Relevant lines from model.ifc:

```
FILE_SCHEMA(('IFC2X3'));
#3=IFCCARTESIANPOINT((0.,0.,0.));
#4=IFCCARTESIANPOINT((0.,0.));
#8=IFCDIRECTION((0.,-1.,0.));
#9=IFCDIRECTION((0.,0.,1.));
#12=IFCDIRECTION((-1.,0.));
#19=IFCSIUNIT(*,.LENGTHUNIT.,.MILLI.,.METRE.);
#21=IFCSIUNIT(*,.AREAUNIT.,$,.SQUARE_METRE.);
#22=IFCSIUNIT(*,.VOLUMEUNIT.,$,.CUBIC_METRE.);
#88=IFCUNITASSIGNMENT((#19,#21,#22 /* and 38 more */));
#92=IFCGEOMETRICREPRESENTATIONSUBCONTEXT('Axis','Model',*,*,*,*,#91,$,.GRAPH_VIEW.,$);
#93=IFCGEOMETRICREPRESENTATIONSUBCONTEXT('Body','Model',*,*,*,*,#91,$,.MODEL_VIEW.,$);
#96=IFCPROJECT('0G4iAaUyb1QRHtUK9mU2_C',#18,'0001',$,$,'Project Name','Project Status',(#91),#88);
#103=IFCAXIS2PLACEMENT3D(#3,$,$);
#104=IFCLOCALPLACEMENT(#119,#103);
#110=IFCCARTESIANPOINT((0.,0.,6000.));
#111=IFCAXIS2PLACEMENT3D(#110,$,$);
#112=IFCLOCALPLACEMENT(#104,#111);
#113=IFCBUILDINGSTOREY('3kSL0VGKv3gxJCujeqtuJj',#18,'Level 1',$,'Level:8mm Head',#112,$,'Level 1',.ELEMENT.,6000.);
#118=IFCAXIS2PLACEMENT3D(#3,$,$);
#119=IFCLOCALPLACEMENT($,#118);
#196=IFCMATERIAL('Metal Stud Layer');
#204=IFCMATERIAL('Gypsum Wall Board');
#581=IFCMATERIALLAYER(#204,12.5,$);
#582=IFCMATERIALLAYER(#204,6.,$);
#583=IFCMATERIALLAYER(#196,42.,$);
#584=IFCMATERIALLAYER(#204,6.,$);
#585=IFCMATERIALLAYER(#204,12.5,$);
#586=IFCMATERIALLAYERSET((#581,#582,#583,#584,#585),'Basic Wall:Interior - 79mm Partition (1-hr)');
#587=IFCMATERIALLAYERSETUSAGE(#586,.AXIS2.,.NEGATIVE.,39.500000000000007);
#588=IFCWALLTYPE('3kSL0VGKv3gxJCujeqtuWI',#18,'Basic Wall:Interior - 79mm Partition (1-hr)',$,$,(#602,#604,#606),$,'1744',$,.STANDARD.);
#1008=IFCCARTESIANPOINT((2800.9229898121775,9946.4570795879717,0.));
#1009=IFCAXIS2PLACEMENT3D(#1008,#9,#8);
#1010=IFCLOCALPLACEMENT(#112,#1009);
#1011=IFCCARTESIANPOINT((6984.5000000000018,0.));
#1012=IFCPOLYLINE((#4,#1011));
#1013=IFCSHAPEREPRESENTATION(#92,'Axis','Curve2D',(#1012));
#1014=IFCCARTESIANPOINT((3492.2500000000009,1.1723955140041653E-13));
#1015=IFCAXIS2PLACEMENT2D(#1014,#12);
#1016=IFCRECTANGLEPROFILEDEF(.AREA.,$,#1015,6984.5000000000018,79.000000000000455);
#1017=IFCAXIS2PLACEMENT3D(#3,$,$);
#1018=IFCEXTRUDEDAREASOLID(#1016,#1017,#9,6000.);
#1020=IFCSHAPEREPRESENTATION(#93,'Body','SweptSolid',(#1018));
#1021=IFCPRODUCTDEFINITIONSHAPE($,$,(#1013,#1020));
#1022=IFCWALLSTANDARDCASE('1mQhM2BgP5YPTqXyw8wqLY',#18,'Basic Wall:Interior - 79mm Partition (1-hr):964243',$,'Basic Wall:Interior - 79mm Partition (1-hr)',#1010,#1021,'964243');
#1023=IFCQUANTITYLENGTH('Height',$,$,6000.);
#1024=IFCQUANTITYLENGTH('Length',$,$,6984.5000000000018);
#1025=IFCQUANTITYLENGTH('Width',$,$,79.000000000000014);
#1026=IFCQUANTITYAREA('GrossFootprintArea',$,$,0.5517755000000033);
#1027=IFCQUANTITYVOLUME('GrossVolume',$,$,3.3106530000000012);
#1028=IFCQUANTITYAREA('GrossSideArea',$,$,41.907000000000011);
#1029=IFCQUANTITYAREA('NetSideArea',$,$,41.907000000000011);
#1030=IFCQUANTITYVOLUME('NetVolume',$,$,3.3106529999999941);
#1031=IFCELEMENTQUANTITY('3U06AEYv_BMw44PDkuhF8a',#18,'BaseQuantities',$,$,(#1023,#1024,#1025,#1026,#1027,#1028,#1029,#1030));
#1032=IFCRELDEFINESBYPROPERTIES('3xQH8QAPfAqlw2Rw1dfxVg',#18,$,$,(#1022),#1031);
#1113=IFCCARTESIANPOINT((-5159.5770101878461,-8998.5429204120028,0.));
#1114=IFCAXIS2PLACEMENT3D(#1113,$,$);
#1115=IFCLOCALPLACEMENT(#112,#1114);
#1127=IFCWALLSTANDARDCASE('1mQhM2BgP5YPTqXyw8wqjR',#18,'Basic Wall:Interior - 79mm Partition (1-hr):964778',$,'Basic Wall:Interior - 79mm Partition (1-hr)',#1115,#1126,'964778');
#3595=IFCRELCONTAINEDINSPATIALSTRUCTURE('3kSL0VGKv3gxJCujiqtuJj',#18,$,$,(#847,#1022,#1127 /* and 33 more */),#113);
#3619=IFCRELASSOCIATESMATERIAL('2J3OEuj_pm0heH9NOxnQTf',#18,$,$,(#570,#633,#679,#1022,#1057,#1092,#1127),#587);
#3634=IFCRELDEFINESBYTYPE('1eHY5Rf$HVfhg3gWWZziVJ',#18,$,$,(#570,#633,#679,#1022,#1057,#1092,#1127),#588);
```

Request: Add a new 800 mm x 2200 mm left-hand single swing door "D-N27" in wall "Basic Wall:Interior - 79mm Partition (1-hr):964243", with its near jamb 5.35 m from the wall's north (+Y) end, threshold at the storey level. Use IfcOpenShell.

```python
import numpy as np
import ifcopenshell
import ifcopenshell.api.feature
import ifcopenshell.api.geometry
import ifcopenshell.api.pset
import ifcopenshell.api.root
import ifcopenshell.api.spatial
import ifcopenshell.api.type
import ifcopenshell.geom
import ifcopenshell.util.element
import ifcopenshell.util.placement
import ifcopenshell.util.representation
import ifcopenshell.util.shape
import ifcopenshell.util.unit

model = ifcopenshell.open("model.ifc")
unit_scale = ifcopenshell.util.unit.calculate_unit_scale(model)
area_scale = ifcopenshell.util.unit.calculate_unit_scale(model, "AREAUNIT")
volume_scale = ifcopenshell.util.unit.calculate_unit_scale(model, "VOLUMEUNIT")
settings = ifcopenshell.geom.settings()


def volume(element):
    """Net volume in cubic metres, openings subtracted."""
    shape = ifcopenshell.geom.create_shape(settings, element)
    return ifcopenshell.util.shape.get_volume(shape.geometry)


wall = model.by_id(1022)
storey = ifcopenshell.util.element.get_container(wall, ifc_class="IfcBuildingStorey")
context = ifcopenshell.util.representation.get_context(model, "Model", "Body", "MODEL_VIEW")
before = volume(wall)

width, height, from_end, sill = 0.8, 2.2, 5.35, 0.0  # metres

# The wall runs along its own X axis, and the end named is its -X end.
wall_shape = ifcopenshell.geom.create_shape(settings, wall)
x, y, z = ifcopenshell.util.shape.get_vertices(wall_shape.geometry).T
start = x.min() + from_end
face, thickness = float(y.min()), float(y.max() - y.min())
wall_matrix = ifcopenshell.util.placement.get_local_placement(wall.ObjectPlacement)
level = ifcopenshell.util.placement.get_local_placement(storey.ObjectPlacement)[2, 3]


def in_wall(x, y):
    """Placement at x, y metres in the wall's axes, at sill height."""
    matrix = wall_matrix.copy()
    matrix[:, 3] = wall_matrix @ np.array([x / unit_scale, y / unit_scale, 0.0, 1.0])
    matrix[2, 3] = level + sill / unit_scale
    return matrix


# Opening: a box that overshoots both wall faces by 50 mm.
opening = ifcopenshell.api.root.create_entity(model, ifc_class="IfcOpeningElement")
box = ifcopenshell.api.geometry.add_wall_representation(
    model, context=context, length=width, height=height, thickness=thickness + 0.1
)
ifcopenshell.api.geometry.assign_representation(model, product=opening, representation=box)
ifcopenshell.api.geometry.edit_object_placement(model, product=opening, matrix=in_wall(start, face - 0.05), is_si=False)
ifcopenshell.api.feature.add_feature(model, feature=opening, element=wall)

door = ifcopenshell.api.root.create_entity(model, ifc_class="IfcDoor", name="D-N27")
door.OverallWidth, door.OverallHeight = width / unit_scale, height / unit_scale
body = ifcopenshell.api.geometry.add_door_representation(
    model,
    context=context,
    overall_width=door.OverallWidth,
    overall_height=door.OverallHeight,
    operation_type="SINGLE_SWING_LEFT",
    lining_properties={"LiningDepth": thickness / unit_scale, "ThresholdDepth": thickness / unit_scale},
)
ifcopenshell.api.geometry.assign_representation(model, product=door, representation=body)
ifcopenshell.api.spatial.assign_container(model, products=[door], relating_structure=storey)
fills = ifcopenshell.api.feature.add_filling(model, opening=opening, element=door)
fills.OwnerHistory = door.OwnerHistory  # required in IFC2X3

# IFC2X3 keeps the operation on the door style.
style = ifcopenshell.api.root.create_entity(model, ifc_class="IfcDoorStyle", name="D-N27")
style.OperationType, style.ConstructionType = "SINGLE_SWING_LEFT", "NOTDEFINED"
style.ParameterTakesPrecedence = style.Sizeable = False
ifcopenshell.api.type.assign_type(model, related_objects=[door], relating_type=style)

# The lining spans the wall, so the door starts at the wall face.
ifcopenshell.api.geometry.edit_object_placement(model, product=door, matrix=in_wall(start, face), is_si=False)

after = volume(wall)

# Update the wall's stored quantities.
qto = model.by_id(ifcopenshell.util.element.get_pset(wall, "BaseQuantities", should_inherit=False)["id"])
ifcopenshell.api.pset.edit_qto(model, qto=qto, properties={
    "NetSideArea": after / thickness / area_scale,
    "NetVolume": after / volume_scale,
})

print(f"wall volume {before:.3f} -> {after:.3f} m3")

model.write("model_v2.ifc")
```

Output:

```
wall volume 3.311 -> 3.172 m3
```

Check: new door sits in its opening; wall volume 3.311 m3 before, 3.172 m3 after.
